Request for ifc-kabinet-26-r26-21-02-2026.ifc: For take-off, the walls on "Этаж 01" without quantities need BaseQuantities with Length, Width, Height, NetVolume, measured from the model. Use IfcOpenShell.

First a look at what the model holds.

```python
import ifcopenshell
import ifcopenshell.util.element
import ifcopenshell.util.unit

model = ifcopenshell.open("ifc-kabinet-26-r26-21-02-2026.ifc")
print(model.schema)
for unit_type in ("LENGTHUNIT", "AREAUNIT", "VOLUMEUNIT"):
    print(unit_type, ifcopenshell.util.unit.calculate_unit_scale(model, unit_type))
storey = next(s for s in model.by_type("IfcBuildingStorey") if s.Name == "Этаж 01")
walls = [e for e in ifcopenshell.util.element.get_decomposition(storey) if e.is_a("IfcWall")]
for e in sorted(walls, key=lambda e: e.id()):
    print(e.id(), e.is_a(), e.Name, list(ifcopenshell.util.element.get_psets(e, qtos_only=True)), sep=" | ")
```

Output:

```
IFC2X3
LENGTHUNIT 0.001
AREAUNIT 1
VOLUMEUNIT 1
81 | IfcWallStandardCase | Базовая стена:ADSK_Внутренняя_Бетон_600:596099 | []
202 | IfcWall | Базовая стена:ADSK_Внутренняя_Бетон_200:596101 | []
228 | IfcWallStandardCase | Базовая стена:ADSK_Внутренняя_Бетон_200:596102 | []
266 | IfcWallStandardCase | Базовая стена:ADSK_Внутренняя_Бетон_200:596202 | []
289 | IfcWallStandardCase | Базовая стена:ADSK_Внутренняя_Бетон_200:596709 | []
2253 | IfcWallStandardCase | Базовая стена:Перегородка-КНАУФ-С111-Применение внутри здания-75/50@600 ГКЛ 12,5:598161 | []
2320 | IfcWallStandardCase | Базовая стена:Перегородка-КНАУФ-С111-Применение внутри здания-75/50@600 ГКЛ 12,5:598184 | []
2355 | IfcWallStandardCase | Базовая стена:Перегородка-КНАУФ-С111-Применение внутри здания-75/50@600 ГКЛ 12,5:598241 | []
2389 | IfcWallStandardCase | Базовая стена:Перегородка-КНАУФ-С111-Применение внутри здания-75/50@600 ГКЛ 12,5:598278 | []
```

```python
import ifcopenshell
import ifcopenshell.api.pset
import ifcopenshell.geom
import ifcopenshell.util.element
import ifcopenshell.util.shape
import ifcopenshell.util.unit

model = ifcopenshell.open("ifc-kabinet-26-r26-21-02-2026.ifc")
unit_scale = ifcopenshell.util.unit.calculate_unit_scale(model)
volume_scale = ifcopenshell.util.unit.calculate_unit_scale(model, "VOLUMEUNIT")
settings = ifcopenshell.geom.settings()

storey = next(s for s in model.by_type("IfcBuildingStorey") if s.Name == "Этаж 01")
walls = [e for e in ifcopenshell.util.element.get_decomposition(storey) if e.is_a("IfcWall")]

for e in sorted(walls, key=lambda e: e.id()):
    if ifcopenshell.util.element.get_psets(e, qtos_only=True, should_inherit=False):
        continue
    # Geometry comes back in metres, in the element's own axes.
    shape = ifcopenshell.geom.create_shape(settings, e)
    values = {
        "Length": ifcopenshell.util.shape.get_x(shape.geometry) / unit_scale,
        "Width": ifcopenshell.util.shape.get_y(shape.geometry) / unit_scale,
        "Height": ifcopenshell.util.shape.get_z(shape.geometry) / unit_scale,
        "NetVolume": ifcopenshell.util.shape.get_volume(shape.geometry) / volume_scale,
    }
    qto = ifcopenshell.api.pset.add_qto(model, product=e, name="BaseQuantities")
    ifcopenshell.api.pset.edit_qto(model, qto=qto, properties=values)
    print(e.id(), {k: round(v, 3) for k, v in values.items()})

model.write("ifc-kabinet-26-r26-21-02-2026_updated.ifc")
```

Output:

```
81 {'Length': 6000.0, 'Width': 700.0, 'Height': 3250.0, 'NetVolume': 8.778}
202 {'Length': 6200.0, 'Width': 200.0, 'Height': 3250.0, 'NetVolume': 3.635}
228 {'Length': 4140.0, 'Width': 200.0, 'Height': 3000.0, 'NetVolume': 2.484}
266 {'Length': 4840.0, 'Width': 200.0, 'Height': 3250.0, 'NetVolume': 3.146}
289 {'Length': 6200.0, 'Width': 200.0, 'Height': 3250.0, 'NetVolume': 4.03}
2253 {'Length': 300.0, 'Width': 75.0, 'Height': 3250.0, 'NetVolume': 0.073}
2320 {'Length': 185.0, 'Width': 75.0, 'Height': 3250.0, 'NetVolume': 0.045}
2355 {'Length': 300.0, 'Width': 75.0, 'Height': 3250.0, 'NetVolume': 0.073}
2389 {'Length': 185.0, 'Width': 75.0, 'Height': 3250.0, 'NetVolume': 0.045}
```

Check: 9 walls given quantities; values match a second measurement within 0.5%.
